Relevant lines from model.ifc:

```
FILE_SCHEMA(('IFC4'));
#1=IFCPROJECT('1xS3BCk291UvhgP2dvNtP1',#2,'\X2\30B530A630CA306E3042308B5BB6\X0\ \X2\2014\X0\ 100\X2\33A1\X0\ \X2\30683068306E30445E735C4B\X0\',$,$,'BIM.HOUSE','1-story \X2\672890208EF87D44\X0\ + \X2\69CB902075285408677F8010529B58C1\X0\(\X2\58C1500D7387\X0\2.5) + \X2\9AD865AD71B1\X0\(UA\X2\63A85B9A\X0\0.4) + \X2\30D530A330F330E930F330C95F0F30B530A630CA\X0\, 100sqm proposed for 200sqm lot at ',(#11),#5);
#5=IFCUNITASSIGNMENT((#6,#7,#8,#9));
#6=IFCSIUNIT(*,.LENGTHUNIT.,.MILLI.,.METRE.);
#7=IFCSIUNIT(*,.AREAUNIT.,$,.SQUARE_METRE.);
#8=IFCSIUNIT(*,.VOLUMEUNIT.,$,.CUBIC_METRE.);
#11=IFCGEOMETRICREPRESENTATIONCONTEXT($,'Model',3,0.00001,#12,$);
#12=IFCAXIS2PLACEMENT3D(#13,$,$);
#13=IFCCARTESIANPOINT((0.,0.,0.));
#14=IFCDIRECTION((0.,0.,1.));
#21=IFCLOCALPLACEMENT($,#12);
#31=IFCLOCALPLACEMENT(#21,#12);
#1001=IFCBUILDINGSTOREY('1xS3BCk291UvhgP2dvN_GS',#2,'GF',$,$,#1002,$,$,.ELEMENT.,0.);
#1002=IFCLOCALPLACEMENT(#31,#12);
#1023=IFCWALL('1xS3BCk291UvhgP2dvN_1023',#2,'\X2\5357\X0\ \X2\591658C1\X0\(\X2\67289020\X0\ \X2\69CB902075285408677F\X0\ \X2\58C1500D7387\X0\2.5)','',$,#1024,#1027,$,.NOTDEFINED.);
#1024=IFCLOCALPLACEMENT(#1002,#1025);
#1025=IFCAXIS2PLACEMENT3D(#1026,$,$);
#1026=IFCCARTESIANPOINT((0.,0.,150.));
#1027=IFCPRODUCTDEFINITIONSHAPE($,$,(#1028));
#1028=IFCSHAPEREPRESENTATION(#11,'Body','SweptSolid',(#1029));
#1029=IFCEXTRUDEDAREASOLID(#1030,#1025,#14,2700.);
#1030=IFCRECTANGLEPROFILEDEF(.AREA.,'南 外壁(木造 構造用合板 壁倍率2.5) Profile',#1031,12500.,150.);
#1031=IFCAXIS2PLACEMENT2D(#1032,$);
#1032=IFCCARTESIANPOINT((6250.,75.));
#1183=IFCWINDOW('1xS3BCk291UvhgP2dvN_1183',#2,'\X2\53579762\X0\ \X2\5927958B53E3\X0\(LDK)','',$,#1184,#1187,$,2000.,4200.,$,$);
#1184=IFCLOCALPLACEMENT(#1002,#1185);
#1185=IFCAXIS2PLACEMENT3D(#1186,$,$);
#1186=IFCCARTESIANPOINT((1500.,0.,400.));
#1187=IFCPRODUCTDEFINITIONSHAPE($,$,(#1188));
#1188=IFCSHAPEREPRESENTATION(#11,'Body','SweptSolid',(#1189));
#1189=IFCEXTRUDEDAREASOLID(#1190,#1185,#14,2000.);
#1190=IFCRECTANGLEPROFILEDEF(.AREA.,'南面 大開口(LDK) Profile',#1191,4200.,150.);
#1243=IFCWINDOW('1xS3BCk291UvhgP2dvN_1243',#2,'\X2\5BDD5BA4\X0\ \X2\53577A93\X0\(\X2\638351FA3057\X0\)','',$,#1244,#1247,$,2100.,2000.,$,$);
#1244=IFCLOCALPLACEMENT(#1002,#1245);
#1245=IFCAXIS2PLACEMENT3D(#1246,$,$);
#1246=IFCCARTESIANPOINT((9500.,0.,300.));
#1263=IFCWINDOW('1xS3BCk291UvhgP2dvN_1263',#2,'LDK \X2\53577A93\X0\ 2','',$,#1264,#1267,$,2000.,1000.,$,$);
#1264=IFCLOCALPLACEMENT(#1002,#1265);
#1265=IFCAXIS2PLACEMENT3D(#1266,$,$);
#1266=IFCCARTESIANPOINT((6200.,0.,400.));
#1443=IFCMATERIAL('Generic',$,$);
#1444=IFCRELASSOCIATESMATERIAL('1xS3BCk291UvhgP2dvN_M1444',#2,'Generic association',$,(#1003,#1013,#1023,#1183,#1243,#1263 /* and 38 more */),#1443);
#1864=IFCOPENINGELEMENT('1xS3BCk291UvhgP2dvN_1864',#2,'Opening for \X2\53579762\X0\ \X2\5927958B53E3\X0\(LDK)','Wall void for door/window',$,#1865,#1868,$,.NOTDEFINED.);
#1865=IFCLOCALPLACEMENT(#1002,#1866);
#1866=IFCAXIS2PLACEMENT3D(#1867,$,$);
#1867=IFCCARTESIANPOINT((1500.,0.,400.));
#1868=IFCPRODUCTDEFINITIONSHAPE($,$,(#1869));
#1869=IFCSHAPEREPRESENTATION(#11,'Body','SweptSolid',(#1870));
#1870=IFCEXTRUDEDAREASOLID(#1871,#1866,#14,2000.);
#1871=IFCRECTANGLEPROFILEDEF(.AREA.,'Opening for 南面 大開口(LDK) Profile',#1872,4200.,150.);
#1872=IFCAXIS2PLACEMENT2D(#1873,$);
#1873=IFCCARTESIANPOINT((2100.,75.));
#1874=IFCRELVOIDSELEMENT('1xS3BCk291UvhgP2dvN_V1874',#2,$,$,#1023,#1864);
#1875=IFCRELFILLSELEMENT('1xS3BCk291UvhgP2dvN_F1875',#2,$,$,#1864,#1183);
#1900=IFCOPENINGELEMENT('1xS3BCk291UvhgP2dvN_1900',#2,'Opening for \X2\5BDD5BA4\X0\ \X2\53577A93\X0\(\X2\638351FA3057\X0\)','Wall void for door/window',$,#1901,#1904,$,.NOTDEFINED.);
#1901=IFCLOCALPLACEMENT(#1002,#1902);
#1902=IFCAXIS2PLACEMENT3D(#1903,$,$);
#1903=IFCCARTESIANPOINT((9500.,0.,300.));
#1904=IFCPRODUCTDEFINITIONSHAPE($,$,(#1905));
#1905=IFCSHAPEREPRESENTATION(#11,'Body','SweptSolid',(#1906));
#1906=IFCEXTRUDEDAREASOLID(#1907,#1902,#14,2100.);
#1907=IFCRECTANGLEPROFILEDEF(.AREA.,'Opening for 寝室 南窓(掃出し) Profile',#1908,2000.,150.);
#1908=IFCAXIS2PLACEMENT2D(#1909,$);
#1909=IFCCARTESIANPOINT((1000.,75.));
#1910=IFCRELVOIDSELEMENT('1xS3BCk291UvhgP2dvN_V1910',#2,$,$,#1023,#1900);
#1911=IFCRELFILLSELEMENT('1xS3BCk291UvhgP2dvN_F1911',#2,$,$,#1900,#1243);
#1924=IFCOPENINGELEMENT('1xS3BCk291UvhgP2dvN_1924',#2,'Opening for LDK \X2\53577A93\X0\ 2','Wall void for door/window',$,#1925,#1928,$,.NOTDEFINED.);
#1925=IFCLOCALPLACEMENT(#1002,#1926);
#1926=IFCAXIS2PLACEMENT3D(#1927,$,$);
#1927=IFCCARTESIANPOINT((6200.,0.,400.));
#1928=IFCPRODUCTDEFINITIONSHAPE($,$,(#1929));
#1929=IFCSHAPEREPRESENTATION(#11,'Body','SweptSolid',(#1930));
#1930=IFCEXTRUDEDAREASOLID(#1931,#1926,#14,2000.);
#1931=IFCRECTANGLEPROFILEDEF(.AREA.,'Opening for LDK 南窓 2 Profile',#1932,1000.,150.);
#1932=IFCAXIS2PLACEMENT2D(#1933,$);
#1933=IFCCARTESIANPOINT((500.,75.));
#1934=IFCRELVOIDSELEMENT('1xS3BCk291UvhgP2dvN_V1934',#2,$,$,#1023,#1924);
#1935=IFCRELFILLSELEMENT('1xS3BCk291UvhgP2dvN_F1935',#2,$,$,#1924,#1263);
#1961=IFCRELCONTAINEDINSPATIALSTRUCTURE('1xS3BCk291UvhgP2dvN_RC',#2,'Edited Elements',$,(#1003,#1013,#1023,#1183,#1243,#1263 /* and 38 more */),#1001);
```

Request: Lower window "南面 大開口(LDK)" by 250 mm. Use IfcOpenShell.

```python
import numpy as np
import ifcopenshell
import ifcopenshell.api.geometry
import ifcopenshell.util.placement
import ifcopenshell.util.unit

model = ifcopenshell.open("model.ifc")
unit_scale = ifcopenshell.util.unit.calculate_unit_scale(model)

window = model.by_guid("1xS3BCk291UvhgP2dvN_1183")
opening = window.FillsVoids[0].RelatingOpeningElement
dz = -250.0

shift = np.array([0.0, 0.0, dz])
# The window is not placed relative to its opening, so move both.
for product in (opening, window):
    matrix = ifcopenshell.util.placement.get_local_placement(product.ObjectPlacement)
    matrix[:3, 3] += shift
    ifcopenshell.api.geometry.edit_object_placement(model, product=product, matrix=matrix, is_si=False)

print(f"moved by {dz * unit_scale:+.3f} m")

model.write("model_updated.ifc")
```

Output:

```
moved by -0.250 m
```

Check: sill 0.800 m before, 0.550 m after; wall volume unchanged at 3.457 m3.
